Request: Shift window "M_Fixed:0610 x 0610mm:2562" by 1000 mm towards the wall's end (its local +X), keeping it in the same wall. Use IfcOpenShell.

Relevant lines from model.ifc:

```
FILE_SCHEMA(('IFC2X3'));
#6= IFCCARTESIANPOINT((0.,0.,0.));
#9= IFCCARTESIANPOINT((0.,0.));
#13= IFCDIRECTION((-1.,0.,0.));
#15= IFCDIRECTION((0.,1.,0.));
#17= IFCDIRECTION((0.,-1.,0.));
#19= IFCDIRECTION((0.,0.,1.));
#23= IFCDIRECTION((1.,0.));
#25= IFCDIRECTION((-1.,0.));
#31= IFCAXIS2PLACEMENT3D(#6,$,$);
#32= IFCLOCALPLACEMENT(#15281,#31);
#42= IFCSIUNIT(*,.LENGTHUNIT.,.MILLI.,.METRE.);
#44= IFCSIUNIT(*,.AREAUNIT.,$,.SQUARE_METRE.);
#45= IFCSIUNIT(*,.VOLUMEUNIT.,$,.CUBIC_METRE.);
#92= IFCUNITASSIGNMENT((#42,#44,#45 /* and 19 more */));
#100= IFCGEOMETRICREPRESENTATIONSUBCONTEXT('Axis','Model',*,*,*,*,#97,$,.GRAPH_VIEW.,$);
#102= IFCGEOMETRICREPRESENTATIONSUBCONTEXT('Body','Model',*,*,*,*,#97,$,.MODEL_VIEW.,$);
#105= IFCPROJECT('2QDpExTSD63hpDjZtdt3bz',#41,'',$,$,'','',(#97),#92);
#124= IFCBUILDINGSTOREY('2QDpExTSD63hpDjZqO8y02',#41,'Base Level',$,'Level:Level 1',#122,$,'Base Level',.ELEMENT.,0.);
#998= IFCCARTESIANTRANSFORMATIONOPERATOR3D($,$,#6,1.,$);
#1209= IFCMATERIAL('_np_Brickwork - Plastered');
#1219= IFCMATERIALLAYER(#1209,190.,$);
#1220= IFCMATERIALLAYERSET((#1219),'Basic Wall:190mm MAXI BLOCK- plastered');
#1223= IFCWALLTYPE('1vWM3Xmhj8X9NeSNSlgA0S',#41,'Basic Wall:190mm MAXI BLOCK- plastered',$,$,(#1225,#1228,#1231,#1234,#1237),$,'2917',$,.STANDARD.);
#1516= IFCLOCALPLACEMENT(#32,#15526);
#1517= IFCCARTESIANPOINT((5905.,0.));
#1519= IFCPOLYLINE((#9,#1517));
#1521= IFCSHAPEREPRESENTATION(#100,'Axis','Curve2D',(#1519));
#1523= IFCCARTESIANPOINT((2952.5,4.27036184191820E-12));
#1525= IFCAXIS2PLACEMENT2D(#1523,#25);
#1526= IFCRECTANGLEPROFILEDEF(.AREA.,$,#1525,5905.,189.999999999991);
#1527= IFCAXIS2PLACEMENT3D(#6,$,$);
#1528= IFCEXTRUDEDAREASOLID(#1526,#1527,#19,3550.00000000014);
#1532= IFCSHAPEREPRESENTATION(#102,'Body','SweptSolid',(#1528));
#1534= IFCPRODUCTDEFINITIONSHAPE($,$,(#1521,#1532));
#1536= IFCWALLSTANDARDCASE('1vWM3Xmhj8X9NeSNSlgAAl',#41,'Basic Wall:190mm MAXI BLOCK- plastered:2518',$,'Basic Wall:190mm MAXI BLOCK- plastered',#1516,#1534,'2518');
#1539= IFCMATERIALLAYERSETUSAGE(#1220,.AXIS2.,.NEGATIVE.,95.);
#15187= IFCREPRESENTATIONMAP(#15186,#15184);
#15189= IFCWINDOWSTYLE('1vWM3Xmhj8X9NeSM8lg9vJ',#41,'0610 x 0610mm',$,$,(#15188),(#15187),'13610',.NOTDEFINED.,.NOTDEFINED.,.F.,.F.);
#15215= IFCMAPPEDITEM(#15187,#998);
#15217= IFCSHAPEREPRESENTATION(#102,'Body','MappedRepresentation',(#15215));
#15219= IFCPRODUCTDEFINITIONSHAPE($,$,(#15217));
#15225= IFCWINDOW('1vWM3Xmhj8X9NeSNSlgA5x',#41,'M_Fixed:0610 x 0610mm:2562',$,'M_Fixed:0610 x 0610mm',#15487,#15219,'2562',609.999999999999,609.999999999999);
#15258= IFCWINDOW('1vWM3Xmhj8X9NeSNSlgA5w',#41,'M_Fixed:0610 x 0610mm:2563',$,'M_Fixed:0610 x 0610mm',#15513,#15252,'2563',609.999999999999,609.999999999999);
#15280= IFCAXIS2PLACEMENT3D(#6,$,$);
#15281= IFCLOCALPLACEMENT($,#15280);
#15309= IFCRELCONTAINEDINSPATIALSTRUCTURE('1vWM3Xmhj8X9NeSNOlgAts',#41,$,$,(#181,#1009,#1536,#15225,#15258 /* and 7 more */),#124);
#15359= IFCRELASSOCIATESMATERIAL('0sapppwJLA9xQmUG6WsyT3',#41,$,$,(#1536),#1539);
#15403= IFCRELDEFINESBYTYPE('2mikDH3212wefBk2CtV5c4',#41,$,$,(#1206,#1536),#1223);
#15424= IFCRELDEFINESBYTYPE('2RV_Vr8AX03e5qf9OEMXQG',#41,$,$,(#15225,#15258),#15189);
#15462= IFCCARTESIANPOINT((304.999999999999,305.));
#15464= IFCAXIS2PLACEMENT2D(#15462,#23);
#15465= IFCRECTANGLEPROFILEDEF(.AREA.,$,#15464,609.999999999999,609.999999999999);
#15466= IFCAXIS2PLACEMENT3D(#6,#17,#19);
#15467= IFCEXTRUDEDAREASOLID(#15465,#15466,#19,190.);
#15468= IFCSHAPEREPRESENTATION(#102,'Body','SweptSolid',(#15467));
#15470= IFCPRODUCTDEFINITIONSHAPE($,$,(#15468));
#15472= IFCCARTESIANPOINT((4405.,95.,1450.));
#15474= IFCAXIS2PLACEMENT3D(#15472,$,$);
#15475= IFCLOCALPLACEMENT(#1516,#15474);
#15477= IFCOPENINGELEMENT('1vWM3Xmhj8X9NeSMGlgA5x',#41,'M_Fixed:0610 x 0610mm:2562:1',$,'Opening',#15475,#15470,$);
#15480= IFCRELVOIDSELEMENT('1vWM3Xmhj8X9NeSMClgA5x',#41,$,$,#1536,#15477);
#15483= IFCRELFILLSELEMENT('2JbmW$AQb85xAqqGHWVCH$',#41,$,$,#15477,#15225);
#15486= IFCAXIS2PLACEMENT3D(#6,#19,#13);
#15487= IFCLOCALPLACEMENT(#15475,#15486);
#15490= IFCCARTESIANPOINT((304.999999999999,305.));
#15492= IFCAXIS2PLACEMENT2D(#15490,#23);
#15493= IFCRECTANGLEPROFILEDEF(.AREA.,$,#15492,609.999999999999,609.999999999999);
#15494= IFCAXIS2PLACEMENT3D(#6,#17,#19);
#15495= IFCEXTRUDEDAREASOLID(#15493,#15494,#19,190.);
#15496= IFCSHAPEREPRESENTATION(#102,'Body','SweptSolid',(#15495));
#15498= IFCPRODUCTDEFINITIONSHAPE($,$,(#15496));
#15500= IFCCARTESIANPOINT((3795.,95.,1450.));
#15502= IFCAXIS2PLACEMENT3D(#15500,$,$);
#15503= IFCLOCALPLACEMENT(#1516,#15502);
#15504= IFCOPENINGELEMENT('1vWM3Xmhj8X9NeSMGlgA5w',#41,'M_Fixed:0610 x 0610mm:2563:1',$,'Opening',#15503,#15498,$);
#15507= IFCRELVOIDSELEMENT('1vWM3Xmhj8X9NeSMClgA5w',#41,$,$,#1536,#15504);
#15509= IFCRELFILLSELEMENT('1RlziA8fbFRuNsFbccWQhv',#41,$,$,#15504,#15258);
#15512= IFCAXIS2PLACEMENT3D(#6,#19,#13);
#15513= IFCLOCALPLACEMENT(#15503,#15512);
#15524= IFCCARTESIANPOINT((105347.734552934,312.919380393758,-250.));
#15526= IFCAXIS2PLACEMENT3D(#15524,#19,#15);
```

```python
import ifcopenshell
import ifcopenshell.api.geometry
import ifcopenshell.util.placement
import ifcopenshell.util.unit

model = ifcopenshell.open("model.ifc")
unit_scale = ifcopenshell.util.unit.calculate_unit_scale(model)

window = model.by_guid("1vWM3Xmhj8X9NeSNSlgA5x")
opening = window.FillsVoids[0].RelatingOpeningElement
wall = opening.VoidsElements[0].RelatingBuildingElement

wall_matrix = ifcopenshell.util.placement.get_local_placement(wall.ObjectPlacement)
shift = wall_matrix[:3, 0] * 1 / unit_scale
before = ifcopenshell.util.placement.get_local_placement(window.ObjectPlacement)[:3, 3].copy()

# The window is placed relative to its opening, so it follows when the opening moves.
matrix = ifcopenshell.util.placement.get_local_placement(opening.ObjectPlacement)
matrix[:3, 3] += shift
ifcopenshell.api.geometry.edit_object_placement(
    model, product=opening, matrix=matrix, is_si=False, should_transform_children=True
)

after = ifcopenshell.util.placement.get_local_placement(window.ObjectPlacement)[:3, 3]
print("window moved by", (after - before).round(3) + 0.0)

model.write("model_rev.ifc")
```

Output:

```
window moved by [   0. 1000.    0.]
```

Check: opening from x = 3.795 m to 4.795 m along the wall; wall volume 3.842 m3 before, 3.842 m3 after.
